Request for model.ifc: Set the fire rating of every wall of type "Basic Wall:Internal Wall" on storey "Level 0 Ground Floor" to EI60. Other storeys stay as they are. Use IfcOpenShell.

First a look at what the model holds.

```python
import ifcopenshell
import ifcopenshell.util.element

model = ifcopenshell.open("model.ifc")
print(model.schema)
storey = next(s for s in model.by_type("IfcBuildingStorey") if s.Name == "Level 0 Ground Floor")
walls = [e for e in ifcopenshell.util.element.get_decomposition(storey) if e.is_a("IfcWall")]
seen = {}
for e in walls:
    element_type = ifcopenshell.util.element.get_type(e)
    key = (element_type.Name if element_type != e and element_type else None, ifcopenshell.util.element.get_pset(e, "Pset_WallCommon", "FireRating"))
    seen[key] = seen.get(key, 0) + 1
for (name, value), count in sorted(seen.items(), key=str):
    print(count, "x", name, "|", value)
```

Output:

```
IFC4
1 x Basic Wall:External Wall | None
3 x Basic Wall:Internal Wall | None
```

```python
import ifcopenshell
import ifcopenshell.api.pset
import ifcopenshell.util.element

model = ifcopenshell.open("model.ifc")

storey = next(s for s in model.by_type("IfcBuildingStorey") if s.Name == "Level 0 Ground Floor")
walls = [e for e in ifcopenshell.util.element.get_decomposition(storey) if e.is_a("IfcWall")]

count = 0
for e in walls:
    element_type = ifcopenshell.util.element.get_type(e)
    if element_type in (None, e) or element_type.Name != "Basic Wall:Internal Wall":
        continue
    # add_pset returns the element's existing set when there is one.
    pset = ifcopenshell.api.pset.add_pset(model, product=e, name="Pset_WallCommon")
    ifcopenshell.api.pset.edit_pset(model, pset=pset, properties={"FireRating": "EI60"})
    count += 1

print(count, "walls updated")

model.write("model_rev.ifc")
```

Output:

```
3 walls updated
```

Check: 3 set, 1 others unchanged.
